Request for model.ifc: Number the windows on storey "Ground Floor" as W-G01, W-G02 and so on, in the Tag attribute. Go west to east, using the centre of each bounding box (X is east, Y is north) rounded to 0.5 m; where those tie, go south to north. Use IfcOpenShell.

First a look at what the model holds.

```python
import ifcopenshell
import ifcopenshell.util.element
import ifcopenshell.util.placement

model = ifcopenshell.open("model.ifc")
print(model.schema)
storey = next(s for s in model.by_type("IfcBuildingStorey") if s.Name == "Ground Floor")
windows = [e for e in ifcopenshell.util.element.get_decomposition(storey) if e.is_a("IfcWindow")]
for e in sorted(windows, key=lambda e: e.id()):
    origin = ifcopenshell.util.placement.get_local_placement(e.ObjectPlacement)[:3, 3]
    print(e.id(), e.Tag, e.Name, origin.round(2) + 0.0, sep=" | ")
```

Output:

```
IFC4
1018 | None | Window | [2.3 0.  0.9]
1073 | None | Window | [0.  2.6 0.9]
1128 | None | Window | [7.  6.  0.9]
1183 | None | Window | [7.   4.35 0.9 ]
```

```python
import ifcopenshell
import ifcopenshell.geom
import ifcopenshell.util.element
import ifcopenshell.util.shape

model = ifcopenshell.open("model.ifc")
settings = ifcopenshell.geom.settings()
settings.set("use-world-coords", True)


def centre(element):
    shape = ifcopenshell.geom.create_shape(settings, element)
    return ifcopenshell.util.shape.get_bbox_centroid(shape.geometry)


storey = next(s for s in model.by_type("IfcBuildingStorey") if s.Name == "Ground Floor")
windows = [e for e in ifcopenshell.util.element.get_decomposition(storey) if e.is_a("IfcWindow")]

# Insertion points can sit at a corner or the storey origin, so sort by the geometry (in metres).
centres = {e: centre(e) for e in windows}
windows.sort(key=lambda e: (round(centres[e][0] / 0.5), centres[e][1]))

for i, e in enumerate(windows, start=1):
    number = f"W-G{i:02d}"
    e.Tag = number
    print(e.id(), number)

model.write("model_updated.ifc")
```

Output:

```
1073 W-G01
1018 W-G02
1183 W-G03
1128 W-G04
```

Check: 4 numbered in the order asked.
